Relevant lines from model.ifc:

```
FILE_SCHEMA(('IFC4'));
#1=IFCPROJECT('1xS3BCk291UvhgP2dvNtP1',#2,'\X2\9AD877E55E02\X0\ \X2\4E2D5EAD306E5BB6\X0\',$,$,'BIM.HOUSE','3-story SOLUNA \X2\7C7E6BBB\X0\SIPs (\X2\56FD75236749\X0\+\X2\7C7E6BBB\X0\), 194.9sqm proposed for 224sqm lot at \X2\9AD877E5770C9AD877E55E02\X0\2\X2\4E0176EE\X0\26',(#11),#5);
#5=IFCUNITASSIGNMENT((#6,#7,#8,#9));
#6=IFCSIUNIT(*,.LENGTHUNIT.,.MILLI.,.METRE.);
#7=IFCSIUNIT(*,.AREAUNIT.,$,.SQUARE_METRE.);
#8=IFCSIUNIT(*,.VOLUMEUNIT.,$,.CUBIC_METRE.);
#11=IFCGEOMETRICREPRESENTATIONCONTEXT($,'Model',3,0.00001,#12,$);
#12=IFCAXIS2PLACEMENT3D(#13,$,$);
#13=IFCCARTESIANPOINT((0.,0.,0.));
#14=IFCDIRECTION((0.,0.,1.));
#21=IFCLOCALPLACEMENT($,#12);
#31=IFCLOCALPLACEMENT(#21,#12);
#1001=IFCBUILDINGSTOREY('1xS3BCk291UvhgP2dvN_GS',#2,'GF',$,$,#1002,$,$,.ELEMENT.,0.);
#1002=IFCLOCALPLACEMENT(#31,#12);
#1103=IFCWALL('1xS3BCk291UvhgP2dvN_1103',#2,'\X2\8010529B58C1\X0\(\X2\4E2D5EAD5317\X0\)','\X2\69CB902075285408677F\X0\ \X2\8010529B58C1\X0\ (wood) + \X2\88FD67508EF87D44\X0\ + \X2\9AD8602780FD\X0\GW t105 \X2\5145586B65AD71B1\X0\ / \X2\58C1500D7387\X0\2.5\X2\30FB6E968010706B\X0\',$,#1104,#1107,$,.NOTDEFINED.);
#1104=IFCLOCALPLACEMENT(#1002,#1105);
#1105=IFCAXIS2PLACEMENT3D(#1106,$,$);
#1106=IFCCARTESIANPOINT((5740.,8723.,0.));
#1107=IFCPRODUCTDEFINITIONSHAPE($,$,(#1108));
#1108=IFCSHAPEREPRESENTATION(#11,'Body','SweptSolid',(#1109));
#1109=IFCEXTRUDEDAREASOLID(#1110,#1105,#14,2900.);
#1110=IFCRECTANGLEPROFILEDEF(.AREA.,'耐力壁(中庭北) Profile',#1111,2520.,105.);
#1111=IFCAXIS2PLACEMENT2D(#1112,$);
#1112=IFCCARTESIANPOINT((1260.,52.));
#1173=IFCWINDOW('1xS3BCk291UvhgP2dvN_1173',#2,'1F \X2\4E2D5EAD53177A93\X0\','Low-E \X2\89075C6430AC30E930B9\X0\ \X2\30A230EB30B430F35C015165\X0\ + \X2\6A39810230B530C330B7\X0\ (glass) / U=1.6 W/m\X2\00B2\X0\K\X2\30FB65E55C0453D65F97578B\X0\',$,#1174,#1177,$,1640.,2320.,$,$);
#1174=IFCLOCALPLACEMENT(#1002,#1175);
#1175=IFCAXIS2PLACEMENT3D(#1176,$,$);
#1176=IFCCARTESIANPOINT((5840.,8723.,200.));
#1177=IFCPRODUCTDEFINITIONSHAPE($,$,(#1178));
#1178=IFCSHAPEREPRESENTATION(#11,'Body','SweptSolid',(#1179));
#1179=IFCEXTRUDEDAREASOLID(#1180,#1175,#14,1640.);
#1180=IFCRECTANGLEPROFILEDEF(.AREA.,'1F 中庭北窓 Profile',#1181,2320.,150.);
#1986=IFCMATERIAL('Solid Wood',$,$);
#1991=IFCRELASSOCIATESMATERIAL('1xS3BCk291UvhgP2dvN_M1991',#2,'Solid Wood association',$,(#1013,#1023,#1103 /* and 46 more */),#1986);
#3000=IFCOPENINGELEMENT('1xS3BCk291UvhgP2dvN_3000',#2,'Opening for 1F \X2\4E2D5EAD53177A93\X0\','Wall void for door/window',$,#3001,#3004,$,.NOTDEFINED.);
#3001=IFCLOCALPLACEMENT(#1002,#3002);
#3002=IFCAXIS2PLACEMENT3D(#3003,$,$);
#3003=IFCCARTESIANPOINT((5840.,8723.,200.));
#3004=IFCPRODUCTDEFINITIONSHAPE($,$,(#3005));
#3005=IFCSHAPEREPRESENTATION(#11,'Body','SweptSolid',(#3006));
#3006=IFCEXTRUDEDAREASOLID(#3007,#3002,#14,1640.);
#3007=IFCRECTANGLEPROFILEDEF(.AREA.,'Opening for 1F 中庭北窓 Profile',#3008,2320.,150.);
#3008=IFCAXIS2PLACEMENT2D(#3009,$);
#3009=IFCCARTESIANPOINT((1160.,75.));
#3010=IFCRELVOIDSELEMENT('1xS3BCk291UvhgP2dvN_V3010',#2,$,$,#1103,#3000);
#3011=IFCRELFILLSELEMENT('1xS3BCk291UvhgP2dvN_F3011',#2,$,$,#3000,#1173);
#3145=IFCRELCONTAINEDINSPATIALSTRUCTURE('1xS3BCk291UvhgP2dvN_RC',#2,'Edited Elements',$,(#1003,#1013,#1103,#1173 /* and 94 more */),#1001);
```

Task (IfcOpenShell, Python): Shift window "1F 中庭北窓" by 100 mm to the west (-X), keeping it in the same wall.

```python
import ifcopenshell
import ifcopenshell.api.geometry
import ifcopenshell.util.placement

model = ifcopenshell.open("model.ifc")

window = model.by_guid("1xS3BCk291UvhgP2dvN_1173")
opening = window.FillsVoids[0].RelatingOpeningElement
wall = opening.VoidsElements[0].RelatingBuildingElement

wall_matrix = ifcopenshell.util.placement.get_local_placement(wall.ObjectPlacement)
shift = wall_matrix[:3, 0] * -100.0
before = ifcopenshell.util.placement.get_local_placement(window.ObjectPlacement)[:3, 3].copy()

# The window is not placed relative to its opening, so move both.
for product in (opening, window):
    matrix = ifcopenshell.util.placement.get_local_placement(product.ObjectPlacement)
    matrix[:3, 3] += shift
    ifcopenshell.api.geometry.edit_object_placement(model, product=product, matrix=matrix, is_si=False)

after = ifcopenshell.util.placement.get_local_placement(window.ObjectPlacement)[:3, 3]
print("window moved by", (after - before).round(3) + 0.0)

model.write("model_edited.ifc")
```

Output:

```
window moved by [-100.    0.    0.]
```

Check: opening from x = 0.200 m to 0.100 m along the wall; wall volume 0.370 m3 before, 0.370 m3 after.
